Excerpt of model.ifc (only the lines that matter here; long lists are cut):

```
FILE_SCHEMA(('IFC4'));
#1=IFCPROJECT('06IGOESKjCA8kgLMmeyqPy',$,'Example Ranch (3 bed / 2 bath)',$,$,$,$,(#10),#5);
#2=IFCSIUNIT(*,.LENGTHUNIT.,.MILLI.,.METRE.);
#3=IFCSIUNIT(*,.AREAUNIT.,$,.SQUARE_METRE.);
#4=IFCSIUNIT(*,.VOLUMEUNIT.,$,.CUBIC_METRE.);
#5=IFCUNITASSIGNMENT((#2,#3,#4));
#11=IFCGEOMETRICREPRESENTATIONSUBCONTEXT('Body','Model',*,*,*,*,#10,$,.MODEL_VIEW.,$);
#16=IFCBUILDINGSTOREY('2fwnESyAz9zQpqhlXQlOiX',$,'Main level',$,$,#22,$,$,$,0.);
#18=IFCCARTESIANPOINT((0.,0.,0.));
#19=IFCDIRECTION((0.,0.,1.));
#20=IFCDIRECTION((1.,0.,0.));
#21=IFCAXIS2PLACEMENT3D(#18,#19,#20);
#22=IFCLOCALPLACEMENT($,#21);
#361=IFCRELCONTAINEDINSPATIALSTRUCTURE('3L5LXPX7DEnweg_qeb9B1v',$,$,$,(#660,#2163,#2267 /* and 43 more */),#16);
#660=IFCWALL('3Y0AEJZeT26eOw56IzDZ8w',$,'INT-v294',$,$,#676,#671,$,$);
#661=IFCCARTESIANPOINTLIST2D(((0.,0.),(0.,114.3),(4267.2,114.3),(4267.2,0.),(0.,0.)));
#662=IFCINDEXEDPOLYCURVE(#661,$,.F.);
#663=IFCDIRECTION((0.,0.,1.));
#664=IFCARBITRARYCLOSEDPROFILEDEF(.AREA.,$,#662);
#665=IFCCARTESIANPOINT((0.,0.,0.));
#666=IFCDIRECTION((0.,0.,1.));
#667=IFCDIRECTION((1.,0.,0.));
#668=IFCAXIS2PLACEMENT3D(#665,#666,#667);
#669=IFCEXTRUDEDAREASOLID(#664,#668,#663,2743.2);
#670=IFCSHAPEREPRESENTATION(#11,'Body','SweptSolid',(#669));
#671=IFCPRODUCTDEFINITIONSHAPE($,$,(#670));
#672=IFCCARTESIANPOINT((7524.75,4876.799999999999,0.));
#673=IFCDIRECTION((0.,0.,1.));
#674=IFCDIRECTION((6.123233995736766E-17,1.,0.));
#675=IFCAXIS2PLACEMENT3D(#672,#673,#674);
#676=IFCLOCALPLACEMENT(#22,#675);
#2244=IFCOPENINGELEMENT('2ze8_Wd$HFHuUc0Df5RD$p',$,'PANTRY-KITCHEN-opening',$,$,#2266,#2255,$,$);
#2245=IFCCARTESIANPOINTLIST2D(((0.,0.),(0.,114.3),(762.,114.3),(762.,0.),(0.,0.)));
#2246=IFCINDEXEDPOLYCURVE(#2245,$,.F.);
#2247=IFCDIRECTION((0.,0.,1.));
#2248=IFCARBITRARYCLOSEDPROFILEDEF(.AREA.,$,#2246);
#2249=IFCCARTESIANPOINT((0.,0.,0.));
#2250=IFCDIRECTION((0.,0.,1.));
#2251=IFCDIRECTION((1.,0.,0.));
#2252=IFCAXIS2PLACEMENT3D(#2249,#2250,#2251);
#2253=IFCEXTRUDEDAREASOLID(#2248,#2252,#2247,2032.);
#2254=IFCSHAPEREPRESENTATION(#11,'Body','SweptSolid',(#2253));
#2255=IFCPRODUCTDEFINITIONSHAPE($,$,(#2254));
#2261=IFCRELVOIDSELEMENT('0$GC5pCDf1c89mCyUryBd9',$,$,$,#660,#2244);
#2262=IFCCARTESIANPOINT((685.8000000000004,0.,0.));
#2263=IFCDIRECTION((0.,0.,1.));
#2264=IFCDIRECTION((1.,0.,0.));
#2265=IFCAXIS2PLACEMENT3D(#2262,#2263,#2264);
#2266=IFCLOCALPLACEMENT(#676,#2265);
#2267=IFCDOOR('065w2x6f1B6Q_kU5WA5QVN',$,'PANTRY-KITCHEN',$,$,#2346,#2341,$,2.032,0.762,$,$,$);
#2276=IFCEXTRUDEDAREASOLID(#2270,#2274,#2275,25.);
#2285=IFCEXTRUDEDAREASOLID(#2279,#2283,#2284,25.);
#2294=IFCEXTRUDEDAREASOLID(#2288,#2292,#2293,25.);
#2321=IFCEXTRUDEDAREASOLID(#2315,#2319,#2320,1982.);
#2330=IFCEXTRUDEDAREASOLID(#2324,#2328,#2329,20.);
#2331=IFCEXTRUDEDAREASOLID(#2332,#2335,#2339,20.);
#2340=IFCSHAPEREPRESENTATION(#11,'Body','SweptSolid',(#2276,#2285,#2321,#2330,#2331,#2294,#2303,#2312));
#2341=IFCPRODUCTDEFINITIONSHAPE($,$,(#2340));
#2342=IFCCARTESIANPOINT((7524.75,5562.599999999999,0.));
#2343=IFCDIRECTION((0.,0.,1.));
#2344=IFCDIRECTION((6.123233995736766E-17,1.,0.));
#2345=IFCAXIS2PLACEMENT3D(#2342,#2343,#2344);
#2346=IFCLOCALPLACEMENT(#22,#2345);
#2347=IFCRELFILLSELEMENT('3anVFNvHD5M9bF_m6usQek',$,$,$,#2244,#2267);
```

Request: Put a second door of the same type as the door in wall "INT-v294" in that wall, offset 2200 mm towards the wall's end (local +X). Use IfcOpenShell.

```python
import ifcopenshell
import ifcopenshell.api.feature
import ifcopenshell.api.geometry
import ifcopenshell.api.root
import ifcopenshell.geom
import ifcopenshell.util.element
import ifcopenshell.util.placement
import ifcopenshell.util.shape
import ifcopenshell.util.unit

model = ifcopenshell.open("model.ifc")
unit_scale = ifcopenshell.util.unit.calculate_unit_scale(model)
settings = ifcopenshell.geom.settings()


def volume(element):
    """Net volume in cubic metres, openings subtracted."""
    shape = ifcopenshell.geom.create_shape(settings, element)
    return ifcopenshell.util.shape.get_volume(shape.geometry)


door = model.by_guid("065w2x6f1B6Q_kU5WA5QVN")
opening = door.FillsVoids[0].RelatingOpeningElement
wall = opening.VoidsElements[0].RelatingBuildingElement
before = volume(wall)
shift = ifcopenshell.util.placement.get_local_placement(wall.ObjectPlacement)[:3, 0] * 2.2 / unit_scale

# copy_class copies the void relationship, type, container and properties, but no geometry.
new_opening = ifcopenshell.api.root.copy_class(model, product=opening)
new_opening.Representation = ifcopenshell.util.element.copy_deep(
    model, opening.Representation, exclude=["IfcGeometricRepresentationContext", "IfcRepresentationMap"]
)
new_door = ifcopenshell.api.root.copy_class(model, product=door)
new_door.Representation = ifcopenshell.util.element.copy_deep(
    model, door.Representation, exclude=["IfcGeometricRepresentationContext", "IfcRepresentationMap"]
)
ifcopenshell.api.feature.add_filling(model, opening=new_opening, element=new_door)

for old, new in ((opening, new_opening), (door, new_door)):
    matrix = ifcopenshell.util.placement.get_local_placement(old.ObjectPlacement)
    matrix[:3, 3] += shift
    ifcopenshell.api.geometry.edit_object_placement(model, product=new, matrix=matrix, is_si=False)

after = volume(wall)

print(f"wall volume {before:.3f} -> {after:.3f} m3")

model.write("model_rev.ifc")
```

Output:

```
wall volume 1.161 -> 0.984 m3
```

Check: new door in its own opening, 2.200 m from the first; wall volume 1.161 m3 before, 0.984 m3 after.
